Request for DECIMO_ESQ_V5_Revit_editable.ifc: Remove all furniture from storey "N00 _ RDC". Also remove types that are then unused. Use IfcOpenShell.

First a look at what the model holds.

```python
import ifcopenshell
import ifcopenshell.util.element

model = ifcopenshell.open("DECIMO_ESQ_V5_Revit_editable.ifc")
print(model.schema)
storey = next(s for s in model.by_type("IfcBuildingStorey") if s.Name == "N00 _ RDC")
furniture = [e for e in ifcopenshell.util.element.get_decomposition(storey) if e.is_a("IfcFurnishingElement")]
seen = {}
for e in furniture:
    element_type = ifcopenshell.util.element.get_type(e)
    name = element_type.Name if element_type not in (None, e) else None
    seen[name] = seen.get(name, 0) + 1
for name, count in sorted(seen.items(), key=str):
    print(count, "x", name)
```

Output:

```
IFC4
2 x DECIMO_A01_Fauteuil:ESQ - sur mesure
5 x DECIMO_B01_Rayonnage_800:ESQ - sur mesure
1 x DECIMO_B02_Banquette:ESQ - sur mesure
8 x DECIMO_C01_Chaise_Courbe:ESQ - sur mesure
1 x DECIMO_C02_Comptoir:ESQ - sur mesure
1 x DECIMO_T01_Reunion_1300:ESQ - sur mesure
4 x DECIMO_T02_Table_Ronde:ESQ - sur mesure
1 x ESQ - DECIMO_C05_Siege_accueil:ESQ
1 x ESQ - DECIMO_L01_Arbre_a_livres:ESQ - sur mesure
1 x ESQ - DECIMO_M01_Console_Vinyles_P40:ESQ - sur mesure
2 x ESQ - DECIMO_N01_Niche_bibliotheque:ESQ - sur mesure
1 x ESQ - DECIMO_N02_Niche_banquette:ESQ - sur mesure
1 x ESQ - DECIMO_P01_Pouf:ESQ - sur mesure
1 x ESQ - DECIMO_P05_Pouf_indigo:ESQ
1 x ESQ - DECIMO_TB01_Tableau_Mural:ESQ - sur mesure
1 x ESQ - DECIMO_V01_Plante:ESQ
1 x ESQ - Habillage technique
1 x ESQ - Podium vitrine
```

```python
import ifcopenshell
import ifcopenshell.api.root
import ifcopenshell.util.element

model = ifcopenshell.open("DECIMO_ESQ_V5_Revit_editable.ifc")

storey = next(s for s in model.by_type("IfcBuildingStorey") if s.Name == "N00 _ RDC")
furniture = [e for e in ifcopenshell.util.element.get_decomposition(storey) if e.is_a("IfcFurnishingElement")]
types = {ifcopenshell.util.element.get_type(e) for e in furniture} - {None, *furniture}

for e in furniture:
    ifcopenshell.api.root.remove_product(model, product=e)
print(len(furniture), "removed")

unused = [t for t in types if not ifcopenshell.util.element.get_types(t)]
for t in unused:
    ifcopenshell.api.root.remove_product(model, product=t)
print(len(unused), "unused types removed")

model.write("DECIMO_ESQ_V5_Revit_editable_rev.ifc")
```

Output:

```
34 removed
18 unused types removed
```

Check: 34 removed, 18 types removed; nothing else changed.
